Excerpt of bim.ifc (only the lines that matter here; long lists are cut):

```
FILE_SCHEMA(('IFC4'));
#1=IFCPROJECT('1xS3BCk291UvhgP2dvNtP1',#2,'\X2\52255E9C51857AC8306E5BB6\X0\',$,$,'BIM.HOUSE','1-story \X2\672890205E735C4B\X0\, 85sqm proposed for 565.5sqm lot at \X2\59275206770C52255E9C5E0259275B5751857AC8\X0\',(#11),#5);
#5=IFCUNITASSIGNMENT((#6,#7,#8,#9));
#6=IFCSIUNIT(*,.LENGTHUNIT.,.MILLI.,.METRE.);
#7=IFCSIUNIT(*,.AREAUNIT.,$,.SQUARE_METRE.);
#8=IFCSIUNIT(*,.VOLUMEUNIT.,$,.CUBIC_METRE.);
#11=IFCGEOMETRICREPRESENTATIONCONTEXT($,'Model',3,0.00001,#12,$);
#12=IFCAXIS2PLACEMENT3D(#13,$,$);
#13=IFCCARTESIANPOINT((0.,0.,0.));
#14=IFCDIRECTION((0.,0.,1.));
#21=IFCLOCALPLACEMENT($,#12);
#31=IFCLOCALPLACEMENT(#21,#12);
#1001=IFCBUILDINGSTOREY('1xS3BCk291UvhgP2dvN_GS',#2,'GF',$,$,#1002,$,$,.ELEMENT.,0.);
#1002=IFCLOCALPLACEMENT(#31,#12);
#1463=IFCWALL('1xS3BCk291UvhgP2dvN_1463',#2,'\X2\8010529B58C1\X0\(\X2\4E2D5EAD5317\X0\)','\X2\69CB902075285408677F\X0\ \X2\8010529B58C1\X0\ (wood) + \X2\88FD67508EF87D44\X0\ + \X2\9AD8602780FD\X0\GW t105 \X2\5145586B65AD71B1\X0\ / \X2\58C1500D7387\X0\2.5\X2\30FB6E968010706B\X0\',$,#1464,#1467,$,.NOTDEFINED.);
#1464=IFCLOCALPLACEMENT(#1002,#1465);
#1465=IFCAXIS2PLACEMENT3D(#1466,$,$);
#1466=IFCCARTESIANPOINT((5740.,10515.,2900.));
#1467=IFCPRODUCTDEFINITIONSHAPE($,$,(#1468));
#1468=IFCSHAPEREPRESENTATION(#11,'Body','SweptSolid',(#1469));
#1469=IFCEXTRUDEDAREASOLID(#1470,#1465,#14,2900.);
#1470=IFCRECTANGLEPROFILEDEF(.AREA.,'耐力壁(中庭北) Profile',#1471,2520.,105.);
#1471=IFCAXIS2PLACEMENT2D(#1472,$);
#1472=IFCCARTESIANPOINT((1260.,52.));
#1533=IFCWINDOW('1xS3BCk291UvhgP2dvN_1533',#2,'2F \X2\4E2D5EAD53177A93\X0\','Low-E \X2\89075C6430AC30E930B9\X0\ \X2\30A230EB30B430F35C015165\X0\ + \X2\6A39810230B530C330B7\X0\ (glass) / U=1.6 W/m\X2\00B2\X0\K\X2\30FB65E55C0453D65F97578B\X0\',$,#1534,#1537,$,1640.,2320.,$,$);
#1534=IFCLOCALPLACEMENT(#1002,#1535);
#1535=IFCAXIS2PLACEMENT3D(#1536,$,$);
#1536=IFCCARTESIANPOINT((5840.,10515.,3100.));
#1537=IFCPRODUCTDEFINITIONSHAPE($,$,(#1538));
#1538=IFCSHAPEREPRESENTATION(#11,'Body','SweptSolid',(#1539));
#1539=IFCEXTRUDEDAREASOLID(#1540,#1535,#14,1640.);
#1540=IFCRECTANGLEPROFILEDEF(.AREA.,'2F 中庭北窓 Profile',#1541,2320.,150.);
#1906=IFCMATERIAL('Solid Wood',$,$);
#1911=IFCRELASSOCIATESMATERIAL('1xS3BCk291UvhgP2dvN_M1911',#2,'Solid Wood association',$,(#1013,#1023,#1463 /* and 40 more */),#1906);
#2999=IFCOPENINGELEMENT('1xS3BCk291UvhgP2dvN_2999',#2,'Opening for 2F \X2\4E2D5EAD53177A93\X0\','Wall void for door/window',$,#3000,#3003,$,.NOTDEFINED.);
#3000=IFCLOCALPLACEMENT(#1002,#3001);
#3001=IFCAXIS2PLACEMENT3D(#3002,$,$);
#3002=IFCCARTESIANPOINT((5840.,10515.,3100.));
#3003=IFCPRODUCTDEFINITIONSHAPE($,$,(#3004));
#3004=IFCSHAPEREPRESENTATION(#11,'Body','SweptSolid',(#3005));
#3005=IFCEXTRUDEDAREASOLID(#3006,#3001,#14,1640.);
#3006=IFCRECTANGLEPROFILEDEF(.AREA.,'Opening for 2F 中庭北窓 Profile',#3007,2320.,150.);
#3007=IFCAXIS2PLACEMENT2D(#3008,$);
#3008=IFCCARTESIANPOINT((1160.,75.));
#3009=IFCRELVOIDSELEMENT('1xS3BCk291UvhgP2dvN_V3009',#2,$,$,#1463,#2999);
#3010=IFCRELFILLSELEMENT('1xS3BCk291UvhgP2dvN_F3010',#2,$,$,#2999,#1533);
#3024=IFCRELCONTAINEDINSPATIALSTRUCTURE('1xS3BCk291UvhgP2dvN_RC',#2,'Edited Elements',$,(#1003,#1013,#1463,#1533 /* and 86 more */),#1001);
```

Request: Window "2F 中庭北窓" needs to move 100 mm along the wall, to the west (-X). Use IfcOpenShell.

```python
import ifcopenshell
import ifcopenshell.api.geometry
import ifcopenshell.util.placement
import ifcopenshell.util.unit

model = ifcopenshell.open("bim.ifc")
unit_scale = ifcopenshell.util.unit.calculate_unit_scale(model)

window = model.by_guid("1xS3BCk291UvhgP2dvN_1533")
opening = window.FillsVoids[0].RelatingOpeningElement
wall = opening.VoidsElements[0].RelatingBuildingElement

wall_matrix = ifcopenshell.util.placement.get_local_placement(wall.ObjectPlacement)
shift = wall_matrix[:3, 0] * -0.1 / unit_scale
before = ifcopenshell.util.placement.get_local_placement(window.ObjectPlacement)[:3, 3].copy()

# The window is not placed relative to its opening, so move both.
for product in (opening, window):
    matrix = ifcopenshell.util.placement.get_local_placement(product.ObjectPlacement)
    matrix[:3, 3] += shift
    ifcopenshell.api.geometry.edit_object_placement(model, product=product, matrix=matrix, is_si=False)

after = ifcopenshell.util.placement.get_local_placement(window.ObjectPlacement)[:3, 3]
print("window moved by", (after - before).round(3) + 0.0)

model.write("bim_edited.ifc")
```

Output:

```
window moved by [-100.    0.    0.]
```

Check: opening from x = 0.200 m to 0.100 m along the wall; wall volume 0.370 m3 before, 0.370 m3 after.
